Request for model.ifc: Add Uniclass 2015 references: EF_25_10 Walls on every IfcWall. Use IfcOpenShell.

First a look at what the model holds.

```python
import ifcopenshell

model = ifcopenshell.open("model.ifc")
print(model.schema)
print("classifications:", [c.Name for c in model.by_type("IfcClassification")])
for ifc_class in ("IfcDoor", "IfcRoof", "IfcStair", "IfcWall", "IfcWindow"):
    print(ifc_class, len(model.by_type(ifc_class)))
```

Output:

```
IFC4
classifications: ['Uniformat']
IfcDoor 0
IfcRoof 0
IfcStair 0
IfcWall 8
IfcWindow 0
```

```python
import ifcopenshell
import ifcopenshell.api.classification

model = ifcopenshell.open("model.ifc")

system = ifcopenshell.api.classification.add_classification(model, classification="Uniclass 2015")

codes = {
    "IfcWall": ("EF_25_10", "Walls"),
}
for ifc_class, (code, name) in codes.items():
    products = model.by_type(ifc_class)
    ifcopenshell.api.classification.add_reference(
        model, products=products, classification=system, identification=code, name=name
    )
    print(code, len(products))

model.write("model_updated.ifc")
```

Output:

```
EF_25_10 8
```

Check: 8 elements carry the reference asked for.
